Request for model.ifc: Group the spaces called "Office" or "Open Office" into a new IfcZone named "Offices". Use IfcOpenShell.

First a look at what the model holds.

```python
import ifcopenshell

model = ifcopenshell.open("model.ifc")
print(model.schema)
seen = {}
for space in model.by_type("IfcSpace"):
    seen[space.LongName] = seen.get(space.LongName, 0) + 1
for name, count in sorted(seen.items(), key=str):
    print(count, "x", name)
print("zones:", [z.Name for z in model.by_type("IfcZone")][:20])
```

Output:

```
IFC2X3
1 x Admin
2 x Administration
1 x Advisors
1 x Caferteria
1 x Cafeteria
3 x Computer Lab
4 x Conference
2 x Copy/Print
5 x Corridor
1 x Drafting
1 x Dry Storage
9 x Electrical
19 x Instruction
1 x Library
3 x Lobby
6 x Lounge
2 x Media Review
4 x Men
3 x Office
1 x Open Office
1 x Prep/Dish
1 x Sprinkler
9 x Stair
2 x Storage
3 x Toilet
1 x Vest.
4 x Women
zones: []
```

```python
import ifcopenshell
import ifcopenshell.api.group
import ifcopenshell.api.root

model = ifcopenshell.open("model.ifc")

names = {"Office", "Open Office"}
spaces = [s for s in model.by_type("IfcSpace") if s.LongName in names]

zone = ifcopenshell.api.root.create_entity(model, ifc_class="IfcZone", name="Offices")
ifcopenshell.api.group.assign_group(model, products=spaces, group=zone)
print(len(spaces), "spaces in", zone.Name)

model.write("model-out.ifc")
```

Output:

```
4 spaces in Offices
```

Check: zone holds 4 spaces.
